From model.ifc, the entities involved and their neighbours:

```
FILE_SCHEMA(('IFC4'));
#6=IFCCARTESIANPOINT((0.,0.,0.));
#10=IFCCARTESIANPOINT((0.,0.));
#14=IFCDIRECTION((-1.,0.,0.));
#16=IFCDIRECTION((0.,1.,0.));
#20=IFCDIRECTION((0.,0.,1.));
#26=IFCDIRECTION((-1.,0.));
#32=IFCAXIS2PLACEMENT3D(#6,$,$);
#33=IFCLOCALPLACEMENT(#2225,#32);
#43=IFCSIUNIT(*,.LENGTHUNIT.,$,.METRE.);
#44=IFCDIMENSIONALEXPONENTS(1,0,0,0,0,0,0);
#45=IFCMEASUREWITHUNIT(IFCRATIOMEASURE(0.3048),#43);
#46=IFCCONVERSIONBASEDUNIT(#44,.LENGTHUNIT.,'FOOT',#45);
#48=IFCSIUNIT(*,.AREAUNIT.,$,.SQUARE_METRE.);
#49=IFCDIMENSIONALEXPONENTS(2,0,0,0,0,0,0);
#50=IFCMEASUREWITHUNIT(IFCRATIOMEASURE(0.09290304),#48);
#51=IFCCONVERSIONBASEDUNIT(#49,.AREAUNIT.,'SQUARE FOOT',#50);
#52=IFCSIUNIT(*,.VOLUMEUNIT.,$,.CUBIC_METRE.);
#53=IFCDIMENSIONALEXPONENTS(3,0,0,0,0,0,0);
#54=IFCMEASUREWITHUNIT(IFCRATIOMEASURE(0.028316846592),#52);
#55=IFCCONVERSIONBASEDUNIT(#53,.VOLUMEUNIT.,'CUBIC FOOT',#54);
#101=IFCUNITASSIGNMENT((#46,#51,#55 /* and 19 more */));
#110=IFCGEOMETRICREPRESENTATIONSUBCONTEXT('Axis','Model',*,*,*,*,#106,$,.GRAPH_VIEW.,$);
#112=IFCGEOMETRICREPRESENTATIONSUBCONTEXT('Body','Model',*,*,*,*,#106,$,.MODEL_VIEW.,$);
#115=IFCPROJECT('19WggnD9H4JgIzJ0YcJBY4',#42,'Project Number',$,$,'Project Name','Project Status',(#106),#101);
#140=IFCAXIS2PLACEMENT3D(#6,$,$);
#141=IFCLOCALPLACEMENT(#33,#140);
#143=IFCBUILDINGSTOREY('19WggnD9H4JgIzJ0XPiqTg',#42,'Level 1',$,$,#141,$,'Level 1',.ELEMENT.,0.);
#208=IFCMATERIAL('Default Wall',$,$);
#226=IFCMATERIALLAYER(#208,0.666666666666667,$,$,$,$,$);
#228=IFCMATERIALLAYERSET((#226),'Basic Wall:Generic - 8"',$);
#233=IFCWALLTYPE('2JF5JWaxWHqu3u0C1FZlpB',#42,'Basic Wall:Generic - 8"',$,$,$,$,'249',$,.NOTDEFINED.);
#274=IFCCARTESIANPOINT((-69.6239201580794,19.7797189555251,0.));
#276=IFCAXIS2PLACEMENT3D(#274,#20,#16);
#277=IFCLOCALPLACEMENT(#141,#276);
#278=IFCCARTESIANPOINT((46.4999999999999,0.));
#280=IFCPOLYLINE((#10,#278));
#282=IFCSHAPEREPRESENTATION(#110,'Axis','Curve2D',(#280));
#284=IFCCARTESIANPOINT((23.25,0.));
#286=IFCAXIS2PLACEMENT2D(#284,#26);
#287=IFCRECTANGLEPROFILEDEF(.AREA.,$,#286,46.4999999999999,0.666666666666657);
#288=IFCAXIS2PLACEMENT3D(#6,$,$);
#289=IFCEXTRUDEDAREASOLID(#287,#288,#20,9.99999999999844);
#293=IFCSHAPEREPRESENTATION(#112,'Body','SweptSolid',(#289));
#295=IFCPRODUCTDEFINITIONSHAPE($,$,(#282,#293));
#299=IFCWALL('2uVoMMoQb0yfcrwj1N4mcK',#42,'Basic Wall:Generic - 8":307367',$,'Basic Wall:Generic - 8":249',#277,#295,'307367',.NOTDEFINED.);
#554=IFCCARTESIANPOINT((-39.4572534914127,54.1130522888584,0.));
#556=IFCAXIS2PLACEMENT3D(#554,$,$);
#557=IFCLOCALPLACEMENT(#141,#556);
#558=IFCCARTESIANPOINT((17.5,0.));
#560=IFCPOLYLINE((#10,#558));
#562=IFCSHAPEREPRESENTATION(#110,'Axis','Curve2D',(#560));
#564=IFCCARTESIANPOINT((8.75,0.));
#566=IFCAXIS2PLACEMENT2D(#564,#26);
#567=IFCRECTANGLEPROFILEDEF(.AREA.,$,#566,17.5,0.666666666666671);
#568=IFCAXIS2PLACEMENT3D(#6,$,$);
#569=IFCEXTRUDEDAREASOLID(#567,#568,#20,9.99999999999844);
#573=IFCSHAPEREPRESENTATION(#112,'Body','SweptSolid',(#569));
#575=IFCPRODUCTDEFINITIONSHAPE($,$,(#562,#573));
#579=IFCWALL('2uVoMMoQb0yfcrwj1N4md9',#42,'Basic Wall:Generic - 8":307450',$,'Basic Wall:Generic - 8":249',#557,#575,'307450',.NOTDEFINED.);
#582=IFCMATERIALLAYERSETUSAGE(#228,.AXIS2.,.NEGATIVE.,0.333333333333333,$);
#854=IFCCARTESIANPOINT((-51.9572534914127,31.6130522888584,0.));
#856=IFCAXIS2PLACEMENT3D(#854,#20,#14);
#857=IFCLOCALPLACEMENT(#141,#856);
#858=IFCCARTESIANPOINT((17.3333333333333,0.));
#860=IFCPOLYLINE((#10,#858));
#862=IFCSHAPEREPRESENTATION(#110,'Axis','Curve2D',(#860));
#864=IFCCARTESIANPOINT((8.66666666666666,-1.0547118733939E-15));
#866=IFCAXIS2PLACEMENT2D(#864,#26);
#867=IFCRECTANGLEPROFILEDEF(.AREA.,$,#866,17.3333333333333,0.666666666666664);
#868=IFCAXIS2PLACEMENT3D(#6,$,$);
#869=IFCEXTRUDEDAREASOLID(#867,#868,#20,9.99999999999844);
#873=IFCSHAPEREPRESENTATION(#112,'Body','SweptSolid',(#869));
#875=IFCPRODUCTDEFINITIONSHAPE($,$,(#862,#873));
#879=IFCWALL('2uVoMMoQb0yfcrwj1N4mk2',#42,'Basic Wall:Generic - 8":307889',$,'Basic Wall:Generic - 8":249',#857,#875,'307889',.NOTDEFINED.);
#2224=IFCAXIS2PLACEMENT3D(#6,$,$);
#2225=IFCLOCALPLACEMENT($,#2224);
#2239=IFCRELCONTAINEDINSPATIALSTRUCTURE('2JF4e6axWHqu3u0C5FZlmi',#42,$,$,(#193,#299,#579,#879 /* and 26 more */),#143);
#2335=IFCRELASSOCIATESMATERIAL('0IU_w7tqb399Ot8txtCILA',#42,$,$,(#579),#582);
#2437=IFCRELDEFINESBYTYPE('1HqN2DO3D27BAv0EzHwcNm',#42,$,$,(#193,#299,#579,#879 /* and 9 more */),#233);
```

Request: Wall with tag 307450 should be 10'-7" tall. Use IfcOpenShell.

```python
import ifcopenshell
import ifcopenshell.geom
import ifcopenshell.util.representation
import ifcopenshell.util.shape
import ifcopenshell.util.unit

model = ifcopenshell.open("model.ifc")
unit_scale = ifcopenshell.util.unit.calculate_unit_scale(model)
settings = ifcopenshell.geom.settings()


def volume(element):
    """Net volume in cubic metres, openings subtracted."""
    shape = ifcopenshell.geom.create_shape(settings, element)
    return ifcopenshell.util.shape.get_volume(shape.geometry)


wall = model.by_guid("2uVoMMoQb0yfcrwj1N4md9")
before = volume(wall)

body = ifcopenshell.util.representation.get_representation(wall, "Model", "Body")
solid = body.Items[0]
old_height = solid.Depth
solid.Depth = 127 * 0.0254 / unit_scale
after = volume(wall)

print(f"height {old_height:g} -> {solid.Depth:g}, volume {before:.3f} -> {after:.3f} m3")

model.write("model_rev.ifc")
```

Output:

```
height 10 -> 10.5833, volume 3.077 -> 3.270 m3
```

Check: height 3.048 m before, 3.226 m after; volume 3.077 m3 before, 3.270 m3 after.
